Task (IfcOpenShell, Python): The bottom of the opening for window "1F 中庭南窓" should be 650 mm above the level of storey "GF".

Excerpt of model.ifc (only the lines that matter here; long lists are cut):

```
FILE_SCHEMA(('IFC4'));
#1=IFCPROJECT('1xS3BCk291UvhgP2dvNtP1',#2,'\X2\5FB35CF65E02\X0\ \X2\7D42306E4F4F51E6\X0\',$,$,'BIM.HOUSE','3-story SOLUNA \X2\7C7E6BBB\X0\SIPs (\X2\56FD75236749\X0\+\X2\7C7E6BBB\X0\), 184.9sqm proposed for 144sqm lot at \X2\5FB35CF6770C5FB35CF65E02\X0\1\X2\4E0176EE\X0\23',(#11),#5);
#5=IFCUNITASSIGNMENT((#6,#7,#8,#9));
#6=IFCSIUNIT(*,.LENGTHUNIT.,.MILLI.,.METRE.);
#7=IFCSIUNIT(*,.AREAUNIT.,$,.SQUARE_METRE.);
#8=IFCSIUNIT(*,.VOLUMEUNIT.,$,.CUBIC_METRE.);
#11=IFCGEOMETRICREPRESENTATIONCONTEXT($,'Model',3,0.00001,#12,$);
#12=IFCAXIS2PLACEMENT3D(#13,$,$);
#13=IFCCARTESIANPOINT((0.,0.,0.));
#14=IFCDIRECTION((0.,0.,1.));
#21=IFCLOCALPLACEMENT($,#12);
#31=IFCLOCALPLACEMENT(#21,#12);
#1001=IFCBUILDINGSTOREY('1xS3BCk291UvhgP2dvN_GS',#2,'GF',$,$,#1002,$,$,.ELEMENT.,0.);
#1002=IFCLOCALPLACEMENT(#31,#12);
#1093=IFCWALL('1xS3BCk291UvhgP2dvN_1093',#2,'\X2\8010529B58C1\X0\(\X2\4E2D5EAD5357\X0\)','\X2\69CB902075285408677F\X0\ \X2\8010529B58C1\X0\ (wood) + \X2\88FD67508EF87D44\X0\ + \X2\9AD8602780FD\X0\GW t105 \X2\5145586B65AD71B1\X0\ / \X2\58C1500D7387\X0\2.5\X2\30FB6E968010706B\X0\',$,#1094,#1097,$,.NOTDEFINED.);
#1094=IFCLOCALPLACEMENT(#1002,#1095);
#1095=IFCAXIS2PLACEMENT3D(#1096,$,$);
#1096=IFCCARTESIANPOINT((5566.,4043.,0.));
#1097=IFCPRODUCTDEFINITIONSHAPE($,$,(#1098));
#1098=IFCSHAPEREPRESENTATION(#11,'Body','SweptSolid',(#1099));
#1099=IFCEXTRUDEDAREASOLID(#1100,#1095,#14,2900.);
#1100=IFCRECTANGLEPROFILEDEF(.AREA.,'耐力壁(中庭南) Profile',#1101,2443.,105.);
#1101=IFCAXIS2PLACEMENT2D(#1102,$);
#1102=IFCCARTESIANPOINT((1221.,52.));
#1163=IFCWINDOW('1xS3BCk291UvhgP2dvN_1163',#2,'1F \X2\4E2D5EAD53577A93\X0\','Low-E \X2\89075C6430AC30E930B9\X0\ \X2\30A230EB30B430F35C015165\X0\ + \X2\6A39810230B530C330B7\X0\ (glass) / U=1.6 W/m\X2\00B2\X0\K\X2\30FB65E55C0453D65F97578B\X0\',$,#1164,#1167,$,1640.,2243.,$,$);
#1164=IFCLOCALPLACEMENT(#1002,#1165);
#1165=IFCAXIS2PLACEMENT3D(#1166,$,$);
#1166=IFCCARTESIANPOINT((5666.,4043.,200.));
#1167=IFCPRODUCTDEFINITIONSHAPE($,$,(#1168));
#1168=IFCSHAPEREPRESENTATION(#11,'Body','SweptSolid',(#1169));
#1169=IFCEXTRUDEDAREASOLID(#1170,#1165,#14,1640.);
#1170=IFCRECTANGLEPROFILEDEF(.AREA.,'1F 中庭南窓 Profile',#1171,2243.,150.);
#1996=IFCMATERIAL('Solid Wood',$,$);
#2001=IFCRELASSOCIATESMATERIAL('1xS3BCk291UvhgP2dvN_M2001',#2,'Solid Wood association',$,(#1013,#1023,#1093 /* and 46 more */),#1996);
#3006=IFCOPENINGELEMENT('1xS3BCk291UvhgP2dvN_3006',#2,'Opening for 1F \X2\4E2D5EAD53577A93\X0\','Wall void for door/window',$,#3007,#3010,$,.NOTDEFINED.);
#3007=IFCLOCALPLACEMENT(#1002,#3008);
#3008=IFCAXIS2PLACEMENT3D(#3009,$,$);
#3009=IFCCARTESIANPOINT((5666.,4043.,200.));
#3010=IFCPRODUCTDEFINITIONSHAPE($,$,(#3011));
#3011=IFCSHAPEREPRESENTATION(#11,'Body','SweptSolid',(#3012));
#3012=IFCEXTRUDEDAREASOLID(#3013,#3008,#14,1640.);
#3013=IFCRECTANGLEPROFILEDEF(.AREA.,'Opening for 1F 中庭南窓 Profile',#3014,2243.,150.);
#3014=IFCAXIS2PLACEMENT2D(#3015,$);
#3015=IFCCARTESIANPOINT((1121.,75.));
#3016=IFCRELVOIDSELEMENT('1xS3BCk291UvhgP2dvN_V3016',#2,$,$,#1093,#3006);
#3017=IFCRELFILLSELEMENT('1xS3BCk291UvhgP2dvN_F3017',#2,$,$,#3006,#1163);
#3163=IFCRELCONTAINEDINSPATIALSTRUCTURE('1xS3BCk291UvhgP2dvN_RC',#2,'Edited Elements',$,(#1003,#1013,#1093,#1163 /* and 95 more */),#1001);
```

```python
import numpy as np
import ifcopenshell
import ifcopenshell.api.geometry
import ifcopenshell.geom
import ifcopenshell.util.element
import ifcopenshell.util.placement
import ifcopenshell.util.shape
import ifcopenshell.util.unit

model = ifcopenshell.open("model.ifc")
unit_scale = ifcopenshell.util.unit.calculate_unit_scale(model)

window = model.by_guid("1xS3BCk291UvhgP2dvN_1163")
opening = window.FillsVoids[0].RelatingOpeningElement
storey = ifcopenshell.util.element.get_container(window, ifc_class="IfcBuildingStorey")
level = ifcopenshell.util.placement.get_local_placement(storey.ObjectPlacement)[2, 3]

# The opening's origin need not be at the sill, so measure its lowest point.
shape = ifcopenshell.geom.create_shape(ifcopenshell.geom.settings(), opening)
bottom = ifcopenshell.util.shape.get_shape_bottom_elevation(shape, shape.geometry) / unit_scale
dz = level + 0.65 / unit_scale - bottom

shift = np.array([0.0, 0.0, dz])
# The window is not placed relative to its opening, so move both.
for product in (opening, window):
    matrix = ifcopenshell.util.placement.get_local_placement(product.ObjectPlacement)
    matrix[:3, 3] += shift
    ifcopenshell.api.geometry.edit_object_placement(model, product=product, matrix=matrix, is_si=False)

print(f"moved by {dz * unit_scale:+.3f} m")

model.write("model_rev.ifc")
```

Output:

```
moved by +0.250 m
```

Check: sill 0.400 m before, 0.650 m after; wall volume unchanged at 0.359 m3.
